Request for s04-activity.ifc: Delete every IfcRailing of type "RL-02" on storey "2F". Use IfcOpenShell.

First a look at what the model holds.

```python
import ifcopenshell
import ifcopenshell.util.element

model = ifcopenshell.open("s04-activity.ifc")
print(model.schema)
storey = next(s for s in model.by_type("IfcBuildingStorey") if s.Name == "2F")
railings = [e for e in ifcopenshell.util.element.get_decomposition(storey) if e.is_a("IfcRailing")]
seen = {}
for e in railings:
    element_type = ifcopenshell.util.element.get_type(e)
    name = element_type.Name if element_type not in (None, e) else None
    seen[name] = seen.get(name, 0) + 1
for name, count in sorted(seen.items(), key=str):
    print(count, "x", name)
```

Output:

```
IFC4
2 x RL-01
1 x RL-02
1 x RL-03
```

```python
import ifcopenshell
import ifcopenshell.api.root
import ifcopenshell.util.element

model = ifcopenshell.open("s04-activity.ifc")

storey = next(s for s in model.by_type("IfcBuildingStorey") if s.Name == "2F")
railings = [e for e in ifcopenshell.util.element.get_decomposition(storey) if e.is_a("IfcRailing")]
targets = [e for e in railings if (t := ifcopenshell.util.element.get_type(e)) not in (None, e) and t.Name == "RL-02"]

for e in targets:
    ifcopenshell.api.root.remove_product(model, product=e)
print(len(targets), "removed")

model.write("s04-activity_edited.ifc")
```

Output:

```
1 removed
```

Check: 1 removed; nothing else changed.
